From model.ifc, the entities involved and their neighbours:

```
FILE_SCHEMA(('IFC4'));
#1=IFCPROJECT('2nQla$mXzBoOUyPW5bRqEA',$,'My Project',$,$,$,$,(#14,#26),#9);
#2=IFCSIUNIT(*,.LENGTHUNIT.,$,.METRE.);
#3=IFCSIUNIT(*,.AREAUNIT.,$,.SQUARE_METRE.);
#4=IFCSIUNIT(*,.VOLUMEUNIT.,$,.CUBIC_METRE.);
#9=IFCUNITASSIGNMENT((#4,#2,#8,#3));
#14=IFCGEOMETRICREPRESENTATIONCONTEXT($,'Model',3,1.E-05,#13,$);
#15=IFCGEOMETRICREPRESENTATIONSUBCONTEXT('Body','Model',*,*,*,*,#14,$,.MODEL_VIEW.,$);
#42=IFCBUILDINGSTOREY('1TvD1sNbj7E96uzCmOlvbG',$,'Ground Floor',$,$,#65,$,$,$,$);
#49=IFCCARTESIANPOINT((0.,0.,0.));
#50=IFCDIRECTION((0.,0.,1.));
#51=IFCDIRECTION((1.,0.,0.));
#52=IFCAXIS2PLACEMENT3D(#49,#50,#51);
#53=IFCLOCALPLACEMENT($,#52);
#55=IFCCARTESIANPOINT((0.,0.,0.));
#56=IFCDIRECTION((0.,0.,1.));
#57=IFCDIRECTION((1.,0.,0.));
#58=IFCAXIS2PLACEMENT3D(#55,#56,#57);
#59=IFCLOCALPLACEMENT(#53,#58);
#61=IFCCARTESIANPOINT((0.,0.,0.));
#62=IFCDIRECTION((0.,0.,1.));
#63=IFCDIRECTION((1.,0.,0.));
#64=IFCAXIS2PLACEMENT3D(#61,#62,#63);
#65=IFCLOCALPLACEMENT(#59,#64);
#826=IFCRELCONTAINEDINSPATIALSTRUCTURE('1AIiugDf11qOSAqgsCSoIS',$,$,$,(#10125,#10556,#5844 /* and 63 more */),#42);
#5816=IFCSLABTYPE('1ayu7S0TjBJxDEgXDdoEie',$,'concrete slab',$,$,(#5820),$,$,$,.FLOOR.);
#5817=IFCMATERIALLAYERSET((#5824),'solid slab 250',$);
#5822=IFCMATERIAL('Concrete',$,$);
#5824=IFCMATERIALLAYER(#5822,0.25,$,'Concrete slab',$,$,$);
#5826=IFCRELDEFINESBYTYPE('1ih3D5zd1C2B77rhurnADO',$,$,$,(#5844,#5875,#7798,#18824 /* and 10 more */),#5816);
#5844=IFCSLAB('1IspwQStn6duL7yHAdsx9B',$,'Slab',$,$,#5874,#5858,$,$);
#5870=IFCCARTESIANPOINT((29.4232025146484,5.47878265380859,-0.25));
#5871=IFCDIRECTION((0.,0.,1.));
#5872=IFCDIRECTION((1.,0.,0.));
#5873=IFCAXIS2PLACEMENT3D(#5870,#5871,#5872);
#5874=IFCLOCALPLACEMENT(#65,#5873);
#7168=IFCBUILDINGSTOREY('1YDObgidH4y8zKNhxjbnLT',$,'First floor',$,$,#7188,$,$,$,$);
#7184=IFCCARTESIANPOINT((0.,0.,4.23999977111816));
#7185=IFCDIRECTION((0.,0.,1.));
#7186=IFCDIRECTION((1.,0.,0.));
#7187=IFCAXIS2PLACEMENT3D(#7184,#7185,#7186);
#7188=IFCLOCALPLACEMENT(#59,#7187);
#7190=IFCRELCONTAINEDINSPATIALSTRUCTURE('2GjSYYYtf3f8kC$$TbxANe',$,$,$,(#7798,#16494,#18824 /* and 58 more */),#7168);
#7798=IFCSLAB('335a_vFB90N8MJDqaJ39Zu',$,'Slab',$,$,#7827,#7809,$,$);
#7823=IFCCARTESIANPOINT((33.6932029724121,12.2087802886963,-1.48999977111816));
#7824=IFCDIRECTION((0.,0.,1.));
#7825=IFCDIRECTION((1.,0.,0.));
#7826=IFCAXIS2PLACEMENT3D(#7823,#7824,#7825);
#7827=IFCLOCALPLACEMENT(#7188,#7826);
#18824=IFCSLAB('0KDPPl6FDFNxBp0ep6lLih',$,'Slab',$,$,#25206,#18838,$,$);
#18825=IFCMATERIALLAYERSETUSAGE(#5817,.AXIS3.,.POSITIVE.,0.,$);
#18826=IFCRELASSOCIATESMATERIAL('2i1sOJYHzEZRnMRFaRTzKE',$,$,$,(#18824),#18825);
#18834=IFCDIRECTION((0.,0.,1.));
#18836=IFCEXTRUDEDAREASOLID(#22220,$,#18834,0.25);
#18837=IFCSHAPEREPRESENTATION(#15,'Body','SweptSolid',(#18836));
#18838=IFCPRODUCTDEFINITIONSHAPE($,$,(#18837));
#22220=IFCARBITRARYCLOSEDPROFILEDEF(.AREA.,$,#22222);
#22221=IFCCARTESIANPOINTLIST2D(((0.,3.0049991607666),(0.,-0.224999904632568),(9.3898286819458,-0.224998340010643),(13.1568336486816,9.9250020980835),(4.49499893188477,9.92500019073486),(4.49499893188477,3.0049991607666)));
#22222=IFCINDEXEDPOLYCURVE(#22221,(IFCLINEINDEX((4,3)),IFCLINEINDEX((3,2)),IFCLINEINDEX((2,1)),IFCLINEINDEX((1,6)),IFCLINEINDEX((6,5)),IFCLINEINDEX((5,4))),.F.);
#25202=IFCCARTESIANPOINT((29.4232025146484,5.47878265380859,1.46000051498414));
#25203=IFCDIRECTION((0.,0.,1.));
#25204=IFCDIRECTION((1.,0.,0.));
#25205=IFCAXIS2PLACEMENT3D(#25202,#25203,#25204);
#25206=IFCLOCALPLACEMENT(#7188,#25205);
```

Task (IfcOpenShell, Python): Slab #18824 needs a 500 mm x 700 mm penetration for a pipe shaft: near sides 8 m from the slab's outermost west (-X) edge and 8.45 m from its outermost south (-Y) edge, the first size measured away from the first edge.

```python
import numpy as np
import ifcopenshell
import ifcopenshell.api.feature
import ifcopenshell.api.geometry
import ifcopenshell.api.root
import ifcopenshell.geom
import ifcopenshell.util.placement
import ifcopenshell.util.representation
import ifcopenshell.util.shape
import ifcopenshell.util.unit

model = ifcopenshell.open("model.ifc")
unit_scale = ifcopenshell.util.unit.calculate_unit_scale(model)
settings = ifcopenshell.geom.settings()


def volume(element):
    """Net volume in cubic metres, openings subtracted."""
    shape = ifcopenshell.geom.create_shape(settings, element)
    return ifcopenshell.util.shape.get_volume(shape.geometry)


slab = model.by_id(18824)
before = volume(slab)

# Extent in the slab's own axes, in metres. The edges named are its -X and -Y sides.
slab_shape = ifcopenshell.geom.create_shape(settings, slab)
vertices = ifcopenshell.util.shape.get_vertices(slab_shape.geometry)
x_min, y_min, bottom = vertices.min(axis=0)
top = vertices[:, 2].max()

opening = ifcopenshell.api.root.create_entity(model, ifc_class="IfcOpeningElement", name="Pipe shaft opening", predefined_type="OPENING")
context = ifcopenshell.util.representation.get_context(model, "Model", "Body", "MODEL_VIEW")
width, depth = 0.5, 0.7
outline = [(0.0, 0.0), (width, 0.0), (width, depth), (0.0, depth), (0.0, 0.0)]
# Overshoot both faces by 50 mm so the cut is clean.
shape = ifcopenshell.api.geometry.add_slab_representation(
    model, context=context, depth=top - bottom + 0.1, polyline=outline
)
ifcopenshell.api.geometry.assign_representation(model, product=opening, representation=shape)

matrix = ifcopenshell.util.placement.get_local_placement(slab.ObjectPlacement)
matrix[:, 3] = matrix @ np.append(np.array([x_min + 8, y_min + 8.45, bottom - 0.05]) / unit_scale, 1.0)
ifcopenshell.api.geometry.edit_object_placement(model, product=opening, matrix=matrix, is_si=False)
ifcopenshell.api.feature.add_feature(model, feature=opening, element=slab)

after = volume(slab)

print(f"slab volume {before:.3f} -> {after:.3f} m3")

model.write("model_v2.ifc")
```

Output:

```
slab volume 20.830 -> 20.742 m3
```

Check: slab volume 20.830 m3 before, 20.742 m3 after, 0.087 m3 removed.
